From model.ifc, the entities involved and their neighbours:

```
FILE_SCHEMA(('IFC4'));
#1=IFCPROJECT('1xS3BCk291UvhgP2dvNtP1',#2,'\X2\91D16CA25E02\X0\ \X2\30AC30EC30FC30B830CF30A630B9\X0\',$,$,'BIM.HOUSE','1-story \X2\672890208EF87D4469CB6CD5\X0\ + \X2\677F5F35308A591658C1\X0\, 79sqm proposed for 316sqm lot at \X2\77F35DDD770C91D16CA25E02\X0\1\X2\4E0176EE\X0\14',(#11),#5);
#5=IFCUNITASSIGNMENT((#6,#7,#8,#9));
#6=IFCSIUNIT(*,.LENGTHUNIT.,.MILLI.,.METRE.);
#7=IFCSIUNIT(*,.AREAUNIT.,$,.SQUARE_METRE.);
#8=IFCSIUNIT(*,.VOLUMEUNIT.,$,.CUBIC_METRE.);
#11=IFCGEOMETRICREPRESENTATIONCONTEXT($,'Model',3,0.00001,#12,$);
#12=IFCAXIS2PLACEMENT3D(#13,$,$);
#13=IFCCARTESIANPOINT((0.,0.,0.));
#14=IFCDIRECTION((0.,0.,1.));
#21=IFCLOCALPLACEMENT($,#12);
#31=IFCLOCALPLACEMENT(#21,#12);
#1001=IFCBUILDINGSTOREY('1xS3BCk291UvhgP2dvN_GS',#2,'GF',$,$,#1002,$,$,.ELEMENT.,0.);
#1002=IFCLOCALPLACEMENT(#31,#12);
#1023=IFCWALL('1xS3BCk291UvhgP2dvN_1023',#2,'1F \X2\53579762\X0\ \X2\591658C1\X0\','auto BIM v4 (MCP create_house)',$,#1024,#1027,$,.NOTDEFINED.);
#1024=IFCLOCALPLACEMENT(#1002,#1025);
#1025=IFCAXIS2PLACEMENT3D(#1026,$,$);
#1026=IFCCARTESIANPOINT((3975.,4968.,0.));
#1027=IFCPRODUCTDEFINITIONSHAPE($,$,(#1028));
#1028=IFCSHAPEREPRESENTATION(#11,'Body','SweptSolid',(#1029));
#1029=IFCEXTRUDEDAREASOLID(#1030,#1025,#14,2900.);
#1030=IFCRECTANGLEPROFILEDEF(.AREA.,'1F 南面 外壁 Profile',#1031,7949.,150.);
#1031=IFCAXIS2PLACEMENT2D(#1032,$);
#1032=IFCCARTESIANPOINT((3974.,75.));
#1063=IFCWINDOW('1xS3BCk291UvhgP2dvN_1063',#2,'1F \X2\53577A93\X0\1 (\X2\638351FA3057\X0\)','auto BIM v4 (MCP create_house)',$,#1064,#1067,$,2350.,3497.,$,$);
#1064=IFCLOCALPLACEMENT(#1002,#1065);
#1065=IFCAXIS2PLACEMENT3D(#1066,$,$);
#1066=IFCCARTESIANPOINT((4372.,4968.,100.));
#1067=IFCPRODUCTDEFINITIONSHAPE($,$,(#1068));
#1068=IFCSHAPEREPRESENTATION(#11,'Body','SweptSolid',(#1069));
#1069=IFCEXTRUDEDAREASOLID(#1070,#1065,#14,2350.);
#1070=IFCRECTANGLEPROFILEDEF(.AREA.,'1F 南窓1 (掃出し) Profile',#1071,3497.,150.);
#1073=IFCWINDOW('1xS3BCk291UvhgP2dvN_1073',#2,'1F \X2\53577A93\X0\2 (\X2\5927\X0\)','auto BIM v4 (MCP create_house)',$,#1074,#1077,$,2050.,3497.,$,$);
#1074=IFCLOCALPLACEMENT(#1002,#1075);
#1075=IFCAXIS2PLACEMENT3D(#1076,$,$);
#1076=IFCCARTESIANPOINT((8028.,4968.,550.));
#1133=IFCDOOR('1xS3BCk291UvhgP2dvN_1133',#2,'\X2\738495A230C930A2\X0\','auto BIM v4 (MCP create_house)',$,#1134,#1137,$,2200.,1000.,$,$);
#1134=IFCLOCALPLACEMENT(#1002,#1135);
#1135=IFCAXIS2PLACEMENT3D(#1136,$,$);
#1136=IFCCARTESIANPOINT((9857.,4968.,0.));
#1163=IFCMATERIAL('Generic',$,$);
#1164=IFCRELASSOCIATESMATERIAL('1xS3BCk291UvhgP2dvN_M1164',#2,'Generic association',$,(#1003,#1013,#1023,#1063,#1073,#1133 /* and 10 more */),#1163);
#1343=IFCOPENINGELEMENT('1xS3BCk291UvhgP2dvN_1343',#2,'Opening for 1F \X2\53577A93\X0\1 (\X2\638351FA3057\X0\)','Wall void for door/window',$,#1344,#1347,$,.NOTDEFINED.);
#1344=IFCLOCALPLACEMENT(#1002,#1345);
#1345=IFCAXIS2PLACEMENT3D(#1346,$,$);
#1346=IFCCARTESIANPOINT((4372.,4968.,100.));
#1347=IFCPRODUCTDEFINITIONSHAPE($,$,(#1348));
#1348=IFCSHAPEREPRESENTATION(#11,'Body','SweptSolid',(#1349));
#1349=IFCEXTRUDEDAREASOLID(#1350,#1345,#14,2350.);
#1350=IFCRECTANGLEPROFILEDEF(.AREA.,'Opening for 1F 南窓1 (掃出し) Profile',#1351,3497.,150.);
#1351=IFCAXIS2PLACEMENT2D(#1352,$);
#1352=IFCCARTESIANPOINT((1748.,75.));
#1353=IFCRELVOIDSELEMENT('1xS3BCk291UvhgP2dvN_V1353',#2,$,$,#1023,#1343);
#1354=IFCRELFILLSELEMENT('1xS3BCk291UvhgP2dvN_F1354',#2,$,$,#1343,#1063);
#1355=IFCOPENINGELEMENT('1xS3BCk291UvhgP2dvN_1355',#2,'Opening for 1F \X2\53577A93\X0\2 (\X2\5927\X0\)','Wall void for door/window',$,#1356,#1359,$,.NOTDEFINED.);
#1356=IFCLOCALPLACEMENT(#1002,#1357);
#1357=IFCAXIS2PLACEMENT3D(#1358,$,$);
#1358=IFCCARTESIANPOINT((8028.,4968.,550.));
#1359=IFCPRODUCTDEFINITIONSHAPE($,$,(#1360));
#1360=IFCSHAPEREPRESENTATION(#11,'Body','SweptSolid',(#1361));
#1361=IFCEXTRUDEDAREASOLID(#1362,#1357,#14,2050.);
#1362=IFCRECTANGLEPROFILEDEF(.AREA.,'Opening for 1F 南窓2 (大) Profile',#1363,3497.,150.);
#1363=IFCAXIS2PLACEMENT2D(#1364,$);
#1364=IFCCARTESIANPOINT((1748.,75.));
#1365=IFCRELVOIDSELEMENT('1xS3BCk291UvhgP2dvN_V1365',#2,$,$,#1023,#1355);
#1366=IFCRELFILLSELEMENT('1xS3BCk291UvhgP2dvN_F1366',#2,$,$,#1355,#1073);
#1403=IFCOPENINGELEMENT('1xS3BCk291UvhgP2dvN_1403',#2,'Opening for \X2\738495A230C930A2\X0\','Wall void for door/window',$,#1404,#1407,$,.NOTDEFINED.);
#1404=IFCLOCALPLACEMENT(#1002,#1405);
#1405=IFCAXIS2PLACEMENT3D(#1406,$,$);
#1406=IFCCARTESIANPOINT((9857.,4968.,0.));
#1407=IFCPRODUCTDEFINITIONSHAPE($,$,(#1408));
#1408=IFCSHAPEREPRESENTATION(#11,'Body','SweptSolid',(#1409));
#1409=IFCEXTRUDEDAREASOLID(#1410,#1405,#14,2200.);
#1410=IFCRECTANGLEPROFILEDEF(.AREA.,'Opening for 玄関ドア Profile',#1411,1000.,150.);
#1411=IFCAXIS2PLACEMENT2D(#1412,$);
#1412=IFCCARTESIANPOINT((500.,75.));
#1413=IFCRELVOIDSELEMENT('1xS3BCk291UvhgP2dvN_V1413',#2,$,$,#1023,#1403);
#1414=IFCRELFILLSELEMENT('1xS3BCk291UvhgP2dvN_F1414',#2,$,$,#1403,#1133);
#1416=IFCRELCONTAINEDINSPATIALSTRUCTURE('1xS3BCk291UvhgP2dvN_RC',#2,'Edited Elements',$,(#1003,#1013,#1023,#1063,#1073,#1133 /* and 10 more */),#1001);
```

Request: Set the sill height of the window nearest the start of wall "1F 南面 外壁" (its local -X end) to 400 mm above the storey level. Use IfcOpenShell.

```python
import numpy as np
import ifcopenshell
import ifcopenshell.api.geometry
import ifcopenshell.geom
import ifcopenshell.util.element
import ifcopenshell.util.placement
import ifcopenshell.util.shape
import ifcopenshell.util.unit

model = ifcopenshell.open("model.ifc")
unit_scale = ifcopenshell.util.unit.calculate_unit_scale(model)

window = model.by_guid("1xS3BCk291UvhgP2dvN_1063")
opening = window.FillsVoids[0].RelatingOpeningElement
storey = ifcopenshell.util.element.get_container(window, ifc_class="IfcBuildingStorey")
level = ifcopenshell.util.placement.get_local_placement(storey.ObjectPlacement)[2, 3]

# The opening's origin need not be at the sill, so measure its lowest point.
shape = ifcopenshell.geom.create_shape(ifcopenshell.geom.settings(), opening)
bottom = ifcopenshell.util.shape.get_shape_bottom_elevation(shape, shape.geometry) / unit_scale
dz = level + 400.0 - bottom

shift = np.array([0.0, 0.0, dz])
# The window is not placed relative to its opening, so move both.
for product in (opening, window):
    matrix = ifcopenshell.util.placement.get_local_placement(product.ObjectPlacement)
    matrix[:3, 3] += shift
    ifcopenshell.api.geometry.edit_object_placement(model, product=product, matrix=matrix, is_si=False)

print(f"moved by {dz * unit_scale:+.3f} m")

model.write("model_edited.ifc")
```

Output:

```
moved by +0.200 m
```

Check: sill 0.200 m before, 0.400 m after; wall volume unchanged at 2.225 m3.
